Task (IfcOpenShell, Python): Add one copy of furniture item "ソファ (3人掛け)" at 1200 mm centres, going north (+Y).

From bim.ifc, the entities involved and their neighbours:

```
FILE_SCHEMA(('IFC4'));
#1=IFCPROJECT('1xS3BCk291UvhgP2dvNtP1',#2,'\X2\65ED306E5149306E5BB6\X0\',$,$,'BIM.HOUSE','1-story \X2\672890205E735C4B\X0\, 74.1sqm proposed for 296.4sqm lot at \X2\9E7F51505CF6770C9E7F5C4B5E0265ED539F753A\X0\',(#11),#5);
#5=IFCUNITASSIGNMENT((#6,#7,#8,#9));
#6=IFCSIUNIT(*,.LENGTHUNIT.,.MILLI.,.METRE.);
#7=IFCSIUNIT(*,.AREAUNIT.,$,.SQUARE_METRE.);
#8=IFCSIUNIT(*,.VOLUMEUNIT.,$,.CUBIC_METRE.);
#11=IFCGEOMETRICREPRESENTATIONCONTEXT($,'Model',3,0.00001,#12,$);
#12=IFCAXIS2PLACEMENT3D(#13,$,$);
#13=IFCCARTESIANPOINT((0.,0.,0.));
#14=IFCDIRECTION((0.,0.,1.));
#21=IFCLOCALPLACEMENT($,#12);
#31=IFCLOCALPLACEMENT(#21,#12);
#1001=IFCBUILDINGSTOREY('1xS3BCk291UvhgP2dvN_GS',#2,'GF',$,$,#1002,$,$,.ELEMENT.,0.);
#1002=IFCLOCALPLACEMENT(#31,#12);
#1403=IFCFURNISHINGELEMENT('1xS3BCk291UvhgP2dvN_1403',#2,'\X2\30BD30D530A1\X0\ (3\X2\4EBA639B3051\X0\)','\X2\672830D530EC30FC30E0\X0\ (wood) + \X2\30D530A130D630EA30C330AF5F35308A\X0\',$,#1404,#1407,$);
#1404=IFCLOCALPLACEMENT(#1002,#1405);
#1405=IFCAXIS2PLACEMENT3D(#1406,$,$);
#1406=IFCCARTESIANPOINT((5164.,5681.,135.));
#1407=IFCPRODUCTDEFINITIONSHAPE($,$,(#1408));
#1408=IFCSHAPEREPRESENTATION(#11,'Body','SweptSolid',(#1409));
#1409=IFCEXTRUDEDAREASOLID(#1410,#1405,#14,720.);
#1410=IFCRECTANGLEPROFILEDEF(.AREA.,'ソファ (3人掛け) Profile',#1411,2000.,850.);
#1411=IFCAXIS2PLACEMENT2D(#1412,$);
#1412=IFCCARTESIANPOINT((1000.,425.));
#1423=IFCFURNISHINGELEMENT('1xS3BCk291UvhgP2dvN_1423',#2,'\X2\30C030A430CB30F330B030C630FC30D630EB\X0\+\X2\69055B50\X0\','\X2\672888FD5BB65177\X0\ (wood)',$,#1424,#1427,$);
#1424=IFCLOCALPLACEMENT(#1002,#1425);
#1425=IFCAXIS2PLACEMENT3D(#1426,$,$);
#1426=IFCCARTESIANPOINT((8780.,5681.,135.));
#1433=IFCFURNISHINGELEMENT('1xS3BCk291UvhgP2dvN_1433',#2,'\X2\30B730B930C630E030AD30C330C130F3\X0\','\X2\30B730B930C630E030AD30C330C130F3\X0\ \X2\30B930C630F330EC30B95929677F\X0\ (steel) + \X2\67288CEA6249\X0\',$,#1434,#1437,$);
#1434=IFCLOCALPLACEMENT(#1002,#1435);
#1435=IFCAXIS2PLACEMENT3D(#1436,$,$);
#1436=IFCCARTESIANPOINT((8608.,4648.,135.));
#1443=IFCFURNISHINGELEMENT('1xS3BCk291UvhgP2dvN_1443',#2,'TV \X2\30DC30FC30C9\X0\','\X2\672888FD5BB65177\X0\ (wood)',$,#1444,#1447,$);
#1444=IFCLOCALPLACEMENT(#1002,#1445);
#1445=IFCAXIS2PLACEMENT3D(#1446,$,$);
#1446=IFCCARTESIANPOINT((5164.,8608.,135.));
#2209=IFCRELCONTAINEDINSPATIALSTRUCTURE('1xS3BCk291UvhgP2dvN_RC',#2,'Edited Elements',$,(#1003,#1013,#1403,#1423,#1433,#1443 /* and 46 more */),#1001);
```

```python
import numpy as np
import ifcopenshell
import ifcopenshell.api.geometry
import ifcopenshell.api.root
import ifcopenshell.util.element
import ifcopenshell.util.placement
import ifcopenshell.util.unit

model = ifcopenshell.open("bim.ifc")
unit_scale = ifcopenshell.util.unit.calculate_unit_scale(model)


def reuse_history(source, copy):
    """copy_class also copies each property set's owner history, people and application; keep the originals."""
    for rel in copy.IsDefinedBy:
        if rel.is_a("IfcRelDefinesByProperties") and (history := rel.RelatingPropertyDefinition.OwnerHistory):
            rel.RelatingPropertyDefinition.OwnerHistory = source.OwnerHistory
            ifcopenshell.util.element.remove_deep2(model, history)


source = model.by_guid("1xS3BCk291UvhgP2dvN_1403")
base = ifcopenshell.util.placement.get_local_placement(source.ObjectPlacement)
step = np.array([0.0, 1.0, 0.0]) * 1.2 / unit_scale

for i in range(1, 2):
    copy = ifcopenshell.api.root.copy_class(model, product=source)
    copy.Representation = ifcopenshell.util.element.copy_deep(
        model, source.Representation, exclude=["IfcGeometricRepresentationContext", "IfcRepresentationMap"]
    )
    reuse_history(source, copy)
    matrix = base.copy()
    matrix[:3, 3] += i * step
    print("added at", matrix[:3, 3].round(3) + 0.0)
    ifcopenshell.api.geometry.edit_object_placement(model, product=copy, matrix=matrix, is_si=False)

model.write("bim_edited.ifc")
```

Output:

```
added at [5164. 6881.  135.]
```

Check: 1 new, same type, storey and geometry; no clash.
